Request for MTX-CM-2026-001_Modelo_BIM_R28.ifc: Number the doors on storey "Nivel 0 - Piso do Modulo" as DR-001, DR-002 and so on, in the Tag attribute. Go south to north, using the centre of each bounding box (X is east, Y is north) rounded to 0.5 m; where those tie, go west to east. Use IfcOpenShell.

First a look at what the model holds.

```python
import ifcopenshell
import ifcopenshell.util.element
import ifcopenshell.util.placement

model = ifcopenshell.open("MTX-CM-2026-001_Modelo_BIM_R28.ifc")
print(model.schema)
storey = next(s for s in model.by_type("IfcBuildingStorey") if s.Name == "Nivel 0 - Piso do Modulo")
doors = [e for e in ifcopenshell.util.element.get_decomposition(storey) if e.is_a("IfcDoor")]
for e in sorted(doors, key=lambda e: e.id()):
    origin = ifcopenshell.util.placement.get_local_placement(e.ObjectPlacement)[:3, 3]
    print(e.id(), e.Tag, e.Name, origin.round(2) + 0.0, sep=" | ")
```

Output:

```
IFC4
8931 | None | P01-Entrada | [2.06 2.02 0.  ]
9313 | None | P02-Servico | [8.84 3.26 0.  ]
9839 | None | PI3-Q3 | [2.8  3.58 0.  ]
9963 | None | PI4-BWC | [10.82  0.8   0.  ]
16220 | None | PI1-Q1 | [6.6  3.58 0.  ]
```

```python
import ifcopenshell
import ifcopenshell.geom
import ifcopenshell.util.element
import ifcopenshell.util.shape

model = ifcopenshell.open("MTX-CM-2026-001_Modelo_BIM_R28.ifc")
settings = ifcopenshell.geom.settings()
settings.set("use-world-coords", True)


def centre(element):
    shape = ifcopenshell.geom.create_shape(settings, element)
    return ifcopenshell.util.shape.get_bbox_centroid(shape.geometry)


storey = next(s for s in model.by_type("IfcBuildingStorey") if s.Name == "Nivel 0 - Piso do Modulo")
doors = [e for e in ifcopenshell.util.element.get_decomposition(storey) if e.is_a("IfcDoor")]

# Insertion points can sit at a corner or the storey origin, so sort by the geometry (in metres).
centres = {e: centre(e) for e in doors}
doors.sort(key=lambda e: (round(centres[e][1] / 0.5), centres[e][0]))

for i, e in enumerate(doors, start=1):
    number = f"DR-0{i:02d}"
    e.Tag = number
    print(e.id(), number)

model.write("MTX-CM-2026-001_Modelo_BIM_R28_updated.ifc")
```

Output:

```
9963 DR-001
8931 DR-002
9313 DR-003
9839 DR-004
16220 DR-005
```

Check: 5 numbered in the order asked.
